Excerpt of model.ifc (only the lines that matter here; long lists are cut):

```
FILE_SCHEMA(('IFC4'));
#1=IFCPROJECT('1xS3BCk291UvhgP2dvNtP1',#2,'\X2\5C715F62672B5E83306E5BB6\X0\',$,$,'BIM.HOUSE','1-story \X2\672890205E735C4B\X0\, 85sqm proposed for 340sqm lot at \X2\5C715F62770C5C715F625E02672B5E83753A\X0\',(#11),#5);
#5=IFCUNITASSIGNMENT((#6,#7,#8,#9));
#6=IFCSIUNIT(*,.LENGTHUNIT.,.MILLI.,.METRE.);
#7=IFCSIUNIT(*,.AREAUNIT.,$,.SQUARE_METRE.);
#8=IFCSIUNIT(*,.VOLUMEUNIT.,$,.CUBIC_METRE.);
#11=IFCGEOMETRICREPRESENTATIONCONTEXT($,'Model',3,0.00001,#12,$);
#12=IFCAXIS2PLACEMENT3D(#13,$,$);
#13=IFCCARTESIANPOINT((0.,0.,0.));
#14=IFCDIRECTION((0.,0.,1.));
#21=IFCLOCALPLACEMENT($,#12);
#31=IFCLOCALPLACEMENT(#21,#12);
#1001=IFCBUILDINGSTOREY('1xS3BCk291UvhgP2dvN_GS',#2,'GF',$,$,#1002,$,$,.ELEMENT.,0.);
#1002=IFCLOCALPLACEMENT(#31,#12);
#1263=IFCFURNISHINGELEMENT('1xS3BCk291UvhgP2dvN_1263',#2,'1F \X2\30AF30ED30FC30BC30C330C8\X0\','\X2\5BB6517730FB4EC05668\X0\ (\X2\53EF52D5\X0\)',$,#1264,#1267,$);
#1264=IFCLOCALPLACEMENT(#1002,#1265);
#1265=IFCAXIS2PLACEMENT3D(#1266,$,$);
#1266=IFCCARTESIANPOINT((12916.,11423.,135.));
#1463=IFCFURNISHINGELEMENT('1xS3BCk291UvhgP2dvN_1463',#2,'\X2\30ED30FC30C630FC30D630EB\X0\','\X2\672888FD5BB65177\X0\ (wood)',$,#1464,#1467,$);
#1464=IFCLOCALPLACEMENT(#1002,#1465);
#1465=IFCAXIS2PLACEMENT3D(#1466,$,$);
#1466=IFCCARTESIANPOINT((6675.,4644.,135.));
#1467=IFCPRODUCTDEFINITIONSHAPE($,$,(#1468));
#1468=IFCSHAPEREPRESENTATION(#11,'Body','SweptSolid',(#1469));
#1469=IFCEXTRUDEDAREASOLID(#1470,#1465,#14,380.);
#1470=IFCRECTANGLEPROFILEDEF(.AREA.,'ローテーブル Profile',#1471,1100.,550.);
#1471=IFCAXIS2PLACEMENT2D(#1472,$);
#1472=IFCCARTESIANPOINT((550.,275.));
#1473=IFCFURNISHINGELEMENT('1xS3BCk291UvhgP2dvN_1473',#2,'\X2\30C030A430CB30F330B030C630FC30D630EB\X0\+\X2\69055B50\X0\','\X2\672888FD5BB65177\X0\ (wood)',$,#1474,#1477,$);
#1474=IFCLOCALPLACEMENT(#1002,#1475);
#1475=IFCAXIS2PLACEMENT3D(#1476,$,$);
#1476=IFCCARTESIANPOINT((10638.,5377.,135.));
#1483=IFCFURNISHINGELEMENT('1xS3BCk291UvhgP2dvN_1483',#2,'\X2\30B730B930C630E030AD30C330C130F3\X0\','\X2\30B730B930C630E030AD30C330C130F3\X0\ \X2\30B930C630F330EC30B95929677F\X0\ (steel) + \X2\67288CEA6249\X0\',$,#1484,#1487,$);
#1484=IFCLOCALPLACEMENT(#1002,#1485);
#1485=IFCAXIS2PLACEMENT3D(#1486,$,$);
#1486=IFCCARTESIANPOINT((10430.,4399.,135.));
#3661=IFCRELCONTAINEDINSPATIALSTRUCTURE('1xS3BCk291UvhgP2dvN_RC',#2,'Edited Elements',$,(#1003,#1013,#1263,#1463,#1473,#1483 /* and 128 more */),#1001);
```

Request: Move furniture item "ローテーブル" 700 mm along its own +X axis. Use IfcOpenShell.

```python
import ifcopenshell
import ifcopenshell.api.geometry
import ifcopenshell.util.placement

model = ifcopenshell.open("model.ifc")

item = model.by_guid("1xS3BCk291UvhgP2dvN_1463")
matrix = ifcopenshell.util.placement.get_local_placement(item.ObjectPlacement)
matrix[:3, 3] += matrix[:3, 0] * 700.0
ifcopenshell.api.geometry.edit_object_placement(model, product=item, matrix=matrix, is_si=False)

print(ifcopenshell.util.placement.get_local_placement(item.ObjectPlacement).round(3) + 0.0)

model.write("model_rev.ifc")
```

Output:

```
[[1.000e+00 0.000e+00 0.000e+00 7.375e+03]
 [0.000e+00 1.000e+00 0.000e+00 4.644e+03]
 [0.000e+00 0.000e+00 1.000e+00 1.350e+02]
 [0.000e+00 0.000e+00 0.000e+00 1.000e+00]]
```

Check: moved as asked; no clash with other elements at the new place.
